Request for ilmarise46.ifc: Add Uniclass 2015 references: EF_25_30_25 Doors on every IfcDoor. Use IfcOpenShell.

First a look at what the model holds.

```python
import ifcopenshell

model = ifcopenshell.open("ilmarise46.ifc")
print(model.schema)
print("classifications:", [c.Name for c in model.by_type("IfcClassification")])
for ifc_class in ("IfcDoor", "IfcRoof", "IfcStair", "IfcWall", "IfcWindow"):
    print(ifc_class, len(model.by_type(ifc_class)))
```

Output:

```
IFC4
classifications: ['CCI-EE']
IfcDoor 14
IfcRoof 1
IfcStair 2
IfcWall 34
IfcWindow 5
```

```python
import ifcopenshell
import ifcopenshell.api.classification

model = ifcopenshell.open("ilmarise46.ifc")

system = ifcopenshell.api.classification.add_classification(model, classification="Uniclass 2015")

codes = {
    "IfcDoor": ("EF_25_30_25", "Doors"),
}
for ifc_class, (code, name) in codes.items():
    products = model.by_type(ifc_class)
    ifcopenshell.api.classification.add_reference(
        model, products=products, classification=system, identification=code, name=name
    )
    print(code, len(products))

model.write("ilmarise46_updated.ifc")
```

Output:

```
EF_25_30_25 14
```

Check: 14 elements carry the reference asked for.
